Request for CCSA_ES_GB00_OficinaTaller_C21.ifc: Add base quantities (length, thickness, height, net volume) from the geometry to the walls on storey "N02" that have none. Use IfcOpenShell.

First a look at what the model holds.

```python
import ifcopenshell
import ifcopenshell.util.element
import ifcopenshell.util.unit

model = ifcopenshell.open("CCSA_ES_GB00_OficinaTaller_C21.ifc")
print(model.schema)
for unit_type in ("LENGTHUNIT", "AREAUNIT", "VOLUMEUNIT"):
    print(unit_type, ifcopenshell.util.unit.calculate_unit_scale(model, unit_type))
storey = next(s for s in model.by_type("IfcBuildingStorey") if s.Name == "N02")
walls = [e for e in ifcopenshell.util.element.get_decomposition(storey) if e.is_a("IfcWall")]
for e in sorted(walls, key=lambda e: e.id()):
    print(e.id(), e.is_a(), e.Name, list(ifcopenshell.util.element.get_psets(e, qtos_only=True)), sep=" | ")
```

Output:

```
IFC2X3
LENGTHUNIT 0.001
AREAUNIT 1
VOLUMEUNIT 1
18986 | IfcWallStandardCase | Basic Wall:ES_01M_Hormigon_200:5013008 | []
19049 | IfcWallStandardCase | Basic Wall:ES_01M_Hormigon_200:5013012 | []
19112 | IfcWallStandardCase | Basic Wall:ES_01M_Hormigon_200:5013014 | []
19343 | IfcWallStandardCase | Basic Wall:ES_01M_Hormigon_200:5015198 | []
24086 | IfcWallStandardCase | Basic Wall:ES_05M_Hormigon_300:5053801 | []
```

```python
import ifcopenshell
import ifcopenshell.api.pset
import ifcopenshell.geom
import ifcopenshell.util.element
import ifcopenshell.util.shape
import ifcopenshell.util.unit

model = ifcopenshell.open("CCSA_ES_GB00_OficinaTaller_C21.ifc")
unit_scale = ifcopenshell.util.unit.calculate_unit_scale(model)
volume_scale = ifcopenshell.util.unit.calculate_unit_scale(model, "VOLUMEUNIT")
settings = ifcopenshell.geom.settings()

storey = next(s for s in model.by_type("IfcBuildingStorey") if s.Name == "N02")
walls = [e for e in ifcopenshell.util.element.get_decomposition(storey) if e.is_a("IfcWall")]

for e in sorted(walls, key=lambda e: e.id()):
    if ifcopenshell.util.element.get_psets(e, qtos_only=True, should_inherit=False):
        continue
    # Geometry comes back in metres, in the element's own axes.
    shape = ifcopenshell.geom.create_shape(settings, e)
    values = {
        "Length": ifcopenshell.util.shape.get_x(shape.geometry) / unit_scale,
        "Width": ifcopenshell.util.shape.get_y(shape.geometry) / unit_scale,
        "Height": ifcopenshell.util.shape.get_z(shape.geometry) / unit_scale,
        "NetVolume": ifcopenshell.util.shape.get_volume(shape.geometry) / volume_scale,
    }
    qto = ifcopenshell.api.pset.add_qto(model, product=e, name="BaseQuantities")
    ifcopenshell.api.pset.edit_qto(model, qto=qto, properties=values)
    print(e.id(), {k: round(v, 3) for k, v in values.items()})

model.write("CCSA_ES_GB00_OficinaTaller_C21-out.ifc")
```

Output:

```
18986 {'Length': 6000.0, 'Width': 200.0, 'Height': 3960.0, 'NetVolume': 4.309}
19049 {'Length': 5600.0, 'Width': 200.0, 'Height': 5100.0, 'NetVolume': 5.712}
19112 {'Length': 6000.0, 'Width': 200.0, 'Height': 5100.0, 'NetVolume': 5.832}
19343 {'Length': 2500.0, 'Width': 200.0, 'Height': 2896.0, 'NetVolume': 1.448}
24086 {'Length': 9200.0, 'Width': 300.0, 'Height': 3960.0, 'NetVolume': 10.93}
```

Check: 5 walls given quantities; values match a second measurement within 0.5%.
